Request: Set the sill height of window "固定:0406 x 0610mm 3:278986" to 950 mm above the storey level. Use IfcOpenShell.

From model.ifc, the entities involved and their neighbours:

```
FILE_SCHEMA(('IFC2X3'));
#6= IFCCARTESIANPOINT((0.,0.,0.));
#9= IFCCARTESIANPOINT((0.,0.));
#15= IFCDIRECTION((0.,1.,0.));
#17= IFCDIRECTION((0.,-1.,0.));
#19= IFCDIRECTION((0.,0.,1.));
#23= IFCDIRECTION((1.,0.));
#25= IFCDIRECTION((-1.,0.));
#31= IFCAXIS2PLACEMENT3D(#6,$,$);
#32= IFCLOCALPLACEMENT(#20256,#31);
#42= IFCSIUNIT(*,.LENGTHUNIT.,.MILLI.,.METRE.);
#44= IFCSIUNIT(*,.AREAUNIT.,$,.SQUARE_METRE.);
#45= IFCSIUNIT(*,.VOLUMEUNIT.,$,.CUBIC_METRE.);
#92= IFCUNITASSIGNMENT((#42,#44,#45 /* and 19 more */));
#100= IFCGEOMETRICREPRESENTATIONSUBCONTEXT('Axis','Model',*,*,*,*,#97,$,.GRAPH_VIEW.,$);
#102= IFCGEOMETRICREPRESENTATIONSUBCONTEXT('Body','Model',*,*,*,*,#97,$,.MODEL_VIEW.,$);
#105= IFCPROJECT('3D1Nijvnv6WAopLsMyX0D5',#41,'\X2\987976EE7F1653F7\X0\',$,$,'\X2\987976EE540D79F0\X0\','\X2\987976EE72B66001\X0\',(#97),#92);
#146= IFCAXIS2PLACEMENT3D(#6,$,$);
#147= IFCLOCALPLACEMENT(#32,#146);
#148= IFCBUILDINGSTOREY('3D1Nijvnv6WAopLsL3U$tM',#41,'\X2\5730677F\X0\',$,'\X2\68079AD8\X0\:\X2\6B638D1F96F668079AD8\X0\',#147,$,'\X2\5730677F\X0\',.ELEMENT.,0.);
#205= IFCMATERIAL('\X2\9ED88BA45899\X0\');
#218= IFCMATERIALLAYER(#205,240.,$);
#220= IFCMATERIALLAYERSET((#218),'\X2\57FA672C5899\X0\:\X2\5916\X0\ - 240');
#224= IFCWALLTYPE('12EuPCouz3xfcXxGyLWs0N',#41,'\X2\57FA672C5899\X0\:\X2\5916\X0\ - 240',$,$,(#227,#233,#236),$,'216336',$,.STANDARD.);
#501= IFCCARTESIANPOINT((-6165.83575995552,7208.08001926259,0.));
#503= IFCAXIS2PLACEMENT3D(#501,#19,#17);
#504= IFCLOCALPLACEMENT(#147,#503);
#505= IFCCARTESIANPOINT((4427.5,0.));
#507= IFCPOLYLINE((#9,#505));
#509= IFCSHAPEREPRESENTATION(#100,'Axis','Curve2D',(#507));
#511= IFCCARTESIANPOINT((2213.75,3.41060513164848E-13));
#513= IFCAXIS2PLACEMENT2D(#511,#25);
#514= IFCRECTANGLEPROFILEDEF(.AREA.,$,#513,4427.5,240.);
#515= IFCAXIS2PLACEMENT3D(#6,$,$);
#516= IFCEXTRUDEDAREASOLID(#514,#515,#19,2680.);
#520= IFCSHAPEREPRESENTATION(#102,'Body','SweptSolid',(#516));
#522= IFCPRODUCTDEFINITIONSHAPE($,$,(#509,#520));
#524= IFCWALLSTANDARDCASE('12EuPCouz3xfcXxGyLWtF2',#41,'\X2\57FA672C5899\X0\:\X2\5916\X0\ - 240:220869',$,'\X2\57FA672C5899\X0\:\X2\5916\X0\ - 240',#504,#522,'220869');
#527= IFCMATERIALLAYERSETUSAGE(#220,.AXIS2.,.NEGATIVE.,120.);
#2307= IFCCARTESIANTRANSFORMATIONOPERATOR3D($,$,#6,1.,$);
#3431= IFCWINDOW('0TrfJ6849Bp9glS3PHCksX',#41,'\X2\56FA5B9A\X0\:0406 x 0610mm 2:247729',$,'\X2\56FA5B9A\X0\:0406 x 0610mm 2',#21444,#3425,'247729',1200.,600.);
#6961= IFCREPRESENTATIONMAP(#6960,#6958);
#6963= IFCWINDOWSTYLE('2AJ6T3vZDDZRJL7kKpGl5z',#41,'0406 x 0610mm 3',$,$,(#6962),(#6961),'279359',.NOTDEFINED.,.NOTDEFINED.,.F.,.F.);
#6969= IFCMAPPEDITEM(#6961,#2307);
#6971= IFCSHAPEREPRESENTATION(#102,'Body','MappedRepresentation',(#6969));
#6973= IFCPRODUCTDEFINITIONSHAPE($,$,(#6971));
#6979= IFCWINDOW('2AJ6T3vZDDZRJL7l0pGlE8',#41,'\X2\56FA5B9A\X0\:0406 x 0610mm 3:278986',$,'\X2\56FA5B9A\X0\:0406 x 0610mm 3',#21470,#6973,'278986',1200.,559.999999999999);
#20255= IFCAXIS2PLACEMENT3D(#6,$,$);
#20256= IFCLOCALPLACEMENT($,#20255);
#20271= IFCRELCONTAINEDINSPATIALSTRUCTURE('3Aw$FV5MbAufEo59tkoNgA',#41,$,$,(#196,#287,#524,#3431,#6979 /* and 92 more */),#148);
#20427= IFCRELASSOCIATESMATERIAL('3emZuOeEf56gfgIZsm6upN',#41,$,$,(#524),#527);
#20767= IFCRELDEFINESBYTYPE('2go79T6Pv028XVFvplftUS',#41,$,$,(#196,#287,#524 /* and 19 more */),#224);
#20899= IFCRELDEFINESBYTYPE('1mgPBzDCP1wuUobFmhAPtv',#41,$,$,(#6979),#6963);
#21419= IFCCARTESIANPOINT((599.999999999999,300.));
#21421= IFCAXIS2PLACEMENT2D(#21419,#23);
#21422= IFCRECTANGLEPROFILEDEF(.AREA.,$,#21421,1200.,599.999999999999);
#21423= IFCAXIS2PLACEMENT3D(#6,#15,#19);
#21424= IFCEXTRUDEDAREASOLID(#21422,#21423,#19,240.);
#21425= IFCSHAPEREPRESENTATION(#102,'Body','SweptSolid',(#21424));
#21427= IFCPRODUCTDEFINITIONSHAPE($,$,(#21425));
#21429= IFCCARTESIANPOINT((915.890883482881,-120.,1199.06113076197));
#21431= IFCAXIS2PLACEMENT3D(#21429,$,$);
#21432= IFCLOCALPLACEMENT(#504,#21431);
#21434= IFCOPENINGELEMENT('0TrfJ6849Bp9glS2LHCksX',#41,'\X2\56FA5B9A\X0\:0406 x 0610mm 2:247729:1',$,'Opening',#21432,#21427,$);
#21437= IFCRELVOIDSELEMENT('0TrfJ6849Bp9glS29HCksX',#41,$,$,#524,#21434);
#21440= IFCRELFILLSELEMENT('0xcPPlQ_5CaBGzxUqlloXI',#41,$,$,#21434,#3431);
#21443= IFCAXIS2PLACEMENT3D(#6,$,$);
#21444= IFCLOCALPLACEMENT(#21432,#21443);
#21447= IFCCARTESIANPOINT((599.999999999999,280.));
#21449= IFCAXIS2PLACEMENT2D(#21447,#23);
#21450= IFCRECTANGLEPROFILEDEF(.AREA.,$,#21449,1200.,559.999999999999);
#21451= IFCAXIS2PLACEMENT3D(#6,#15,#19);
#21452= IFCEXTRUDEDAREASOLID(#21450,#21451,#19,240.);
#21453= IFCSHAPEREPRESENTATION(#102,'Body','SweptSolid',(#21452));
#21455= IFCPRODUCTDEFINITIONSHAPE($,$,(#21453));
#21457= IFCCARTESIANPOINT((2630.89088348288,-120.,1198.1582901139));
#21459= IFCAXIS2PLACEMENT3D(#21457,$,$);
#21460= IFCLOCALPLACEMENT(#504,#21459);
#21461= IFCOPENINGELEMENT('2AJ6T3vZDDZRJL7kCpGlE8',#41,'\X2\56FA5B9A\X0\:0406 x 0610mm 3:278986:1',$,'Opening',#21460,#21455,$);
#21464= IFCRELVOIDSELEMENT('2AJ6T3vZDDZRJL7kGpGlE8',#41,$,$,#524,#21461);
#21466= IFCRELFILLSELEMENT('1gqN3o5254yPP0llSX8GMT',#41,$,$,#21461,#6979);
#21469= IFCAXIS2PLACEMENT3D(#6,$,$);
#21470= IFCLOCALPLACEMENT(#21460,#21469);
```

```python
import numpy as np
import ifcopenshell
import ifcopenshell.api.geometry
import ifcopenshell.geom
import ifcopenshell.util.element
import ifcopenshell.util.placement
import ifcopenshell.util.shape
import ifcopenshell.util.unit

model = ifcopenshell.open("model.ifc")
unit_scale = ifcopenshell.util.unit.calculate_unit_scale(model)

window = model.by_guid("2AJ6T3vZDDZRJL7l0pGlE8")
opening = window.FillsVoids[0].RelatingOpeningElement
storey = ifcopenshell.util.element.get_container(window, ifc_class="IfcBuildingStorey")
level = ifcopenshell.util.placement.get_local_placement(storey.ObjectPlacement)[2, 3]

# The opening's origin need not be at the sill, so measure its lowest point.
shape = ifcopenshell.geom.create_shape(ifcopenshell.geom.settings(), opening)
bottom = ifcopenshell.util.shape.get_shape_bottom_elevation(shape, shape.geometry) / unit_scale
dz = level + 950.0 - bottom

shift = np.array([0.0, 0.0, dz])
# The window is placed relative to its opening, so it follows when the opening moves.
matrix = ifcopenshell.util.placement.get_local_placement(opening.ObjectPlacement)
matrix[:3, 3] += shift
ifcopenshell.api.geometry.edit_object_placement(
    model, product=opening, matrix=matrix, is_si=False, should_transform_children=True
)

print(f"moved by {dz * unit_scale:+.3f} m")

model.write("model-out.ifc")
```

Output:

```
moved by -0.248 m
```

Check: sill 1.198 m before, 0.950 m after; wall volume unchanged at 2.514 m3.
